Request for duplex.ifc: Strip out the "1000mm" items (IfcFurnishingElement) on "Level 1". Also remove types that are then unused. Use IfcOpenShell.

First a look at what the model holds.

```python
import ifcopenshell
import ifcopenshell.util.element

model = ifcopenshell.open("duplex.ifc")
print(model.schema)
storey = next(s for s in model.by_type("IfcBuildingStorey") if s.Name == "Level 1")
furniture = [e for e in ifcopenshell.util.element.get_decomposition(storey) if e.is_a("IfcFurnishingElement")]
seen = {}
for e in furniture:
    element_type = ifcopenshell.util.element.get_type(e)
    name = element_type.Name if element_type not in (None, e) else None
    seen[name] = seen.get(name, 0) + 1
for name, count in sorted(seen.items(), key=str):
    print(count, "x", name)
```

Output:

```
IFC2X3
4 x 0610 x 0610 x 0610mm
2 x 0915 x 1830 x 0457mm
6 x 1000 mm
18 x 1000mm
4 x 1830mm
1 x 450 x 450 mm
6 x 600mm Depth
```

```python
import ifcopenshell
import ifcopenshell.api.root
import ifcopenshell.util.element

model = ifcopenshell.open("duplex.ifc")

storey = next(s for s in model.by_type("IfcBuildingStorey") if s.Name == "Level 1")
furniture = [e for e in ifcopenshell.util.element.get_decomposition(storey) if e.is_a("IfcFurnishingElement")]
targets = [e for e in furniture if (t := ifcopenshell.util.element.get_type(e)) not in (None, e) and t.Name == "1000mm"]
types = {ifcopenshell.util.element.get_type(e) for e in targets} - {None, *targets}

for e in targets:
    ifcopenshell.api.root.remove_product(model, product=e)
print(len(targets), "removed")

unused = [t for t in types if not ifcopenshell.util.element.get_types(t)]
for t in unused:
    ifcopenshell.api.root.remove_product(model, product=t)
print(len(unused), "unused types removed")

model.write("duplex_rev.ifc")
```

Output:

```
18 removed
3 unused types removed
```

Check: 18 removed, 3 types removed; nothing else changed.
